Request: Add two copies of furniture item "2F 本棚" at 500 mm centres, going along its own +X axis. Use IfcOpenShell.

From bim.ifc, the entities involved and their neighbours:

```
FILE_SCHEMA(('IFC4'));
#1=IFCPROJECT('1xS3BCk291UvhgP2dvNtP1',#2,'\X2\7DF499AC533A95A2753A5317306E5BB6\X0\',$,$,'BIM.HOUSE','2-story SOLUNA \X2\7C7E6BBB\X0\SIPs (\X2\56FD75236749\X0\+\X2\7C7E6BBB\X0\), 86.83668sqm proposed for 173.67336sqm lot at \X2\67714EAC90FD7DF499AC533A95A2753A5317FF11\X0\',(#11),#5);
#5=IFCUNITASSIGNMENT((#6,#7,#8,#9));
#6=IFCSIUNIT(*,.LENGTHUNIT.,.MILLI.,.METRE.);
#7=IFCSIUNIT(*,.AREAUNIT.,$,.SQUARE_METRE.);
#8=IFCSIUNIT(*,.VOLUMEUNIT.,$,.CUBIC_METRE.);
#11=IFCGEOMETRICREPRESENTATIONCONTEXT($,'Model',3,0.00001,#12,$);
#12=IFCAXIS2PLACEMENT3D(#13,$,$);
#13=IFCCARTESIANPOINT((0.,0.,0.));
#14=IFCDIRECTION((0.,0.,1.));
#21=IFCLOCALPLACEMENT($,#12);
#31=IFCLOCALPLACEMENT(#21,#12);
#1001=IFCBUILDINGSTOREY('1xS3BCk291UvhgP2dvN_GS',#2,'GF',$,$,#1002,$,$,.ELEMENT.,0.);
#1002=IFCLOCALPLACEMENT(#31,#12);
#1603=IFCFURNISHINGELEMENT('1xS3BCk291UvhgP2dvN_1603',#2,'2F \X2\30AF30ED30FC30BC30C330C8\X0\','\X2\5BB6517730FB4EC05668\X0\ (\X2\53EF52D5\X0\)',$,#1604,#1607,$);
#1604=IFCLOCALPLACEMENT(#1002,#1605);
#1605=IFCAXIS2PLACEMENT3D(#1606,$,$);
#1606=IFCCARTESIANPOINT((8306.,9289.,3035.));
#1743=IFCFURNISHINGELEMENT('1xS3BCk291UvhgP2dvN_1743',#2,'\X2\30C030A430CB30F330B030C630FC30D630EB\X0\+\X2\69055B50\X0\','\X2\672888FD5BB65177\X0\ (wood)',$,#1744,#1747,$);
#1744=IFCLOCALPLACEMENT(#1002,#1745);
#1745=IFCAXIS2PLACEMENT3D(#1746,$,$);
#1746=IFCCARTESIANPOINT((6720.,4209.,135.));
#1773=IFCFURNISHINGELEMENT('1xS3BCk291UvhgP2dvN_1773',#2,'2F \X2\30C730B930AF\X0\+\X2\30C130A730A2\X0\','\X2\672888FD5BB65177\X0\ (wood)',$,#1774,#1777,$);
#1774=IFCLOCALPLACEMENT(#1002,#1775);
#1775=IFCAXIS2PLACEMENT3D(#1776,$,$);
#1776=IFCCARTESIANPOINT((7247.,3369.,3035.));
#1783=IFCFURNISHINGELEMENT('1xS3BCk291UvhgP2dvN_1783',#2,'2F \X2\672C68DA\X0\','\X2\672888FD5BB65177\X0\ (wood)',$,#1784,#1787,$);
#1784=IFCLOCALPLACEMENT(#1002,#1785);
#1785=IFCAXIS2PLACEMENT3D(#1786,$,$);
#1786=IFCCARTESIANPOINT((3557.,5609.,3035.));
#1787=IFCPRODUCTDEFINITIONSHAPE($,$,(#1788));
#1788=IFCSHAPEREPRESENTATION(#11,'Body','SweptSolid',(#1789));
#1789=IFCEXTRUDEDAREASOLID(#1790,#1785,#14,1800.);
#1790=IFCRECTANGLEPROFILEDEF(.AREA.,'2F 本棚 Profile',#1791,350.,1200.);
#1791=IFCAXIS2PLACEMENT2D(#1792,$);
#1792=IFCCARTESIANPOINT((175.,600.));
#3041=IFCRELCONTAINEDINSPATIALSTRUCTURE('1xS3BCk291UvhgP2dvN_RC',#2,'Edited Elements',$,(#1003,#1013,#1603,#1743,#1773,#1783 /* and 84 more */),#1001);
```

```python
import ifcopenshell
import ifcopenshell.api.geometry
import ifcopenshell.api.root
import ifcopenshell.util.element
import ifcopenshell.util.placement
import ifcopenshell.util.unit

model = ifcopenshell.open("bim.ifc")
unit_scale = ifcopenshell.util.unit.calculate_unit_scale(model)


def reuse_history(source, copy):
    """copy_class also copies each property set's owner history, people and application; keep the originals."""
    for rel in copy.IsDefinedBy:
        if rel.is_a("IfcRelDefinesByProperties") and (history := rel.RelatingPropertyDefinition.OwnerHistory):
            rel.RelatingPropertyDefinition.OwnerHistory = source.OwnerHistory
            ifcopenshell.util.element.remove_deep2(model, history)


source = model.by_guid("1xS3BCk291UvhgP2dvN_1783")
base = ifcopenshell.util.placement.get_local_placement(source.ObjectPlacement)
step = base[:3, 0] * 0.5 / unit_scale

for i in range(1, 3):
    copy = ifcopenshell.api.root.copy_class(model, product=source)
    copy.Representation = ifcopenshell.util.element.copy_deep(
        model, source.Representation, exclude=["IfcGeometricRepresentationContext", "IfcRepresentationMap"]
    )
    reuse_history(source, copy)
    matrix = base.copy()
    matrix[:3, 3] += i * step
    print("added at", matrix[:3, 3].round(3) + 0.0)
    ifcopenshell.api.geometry.edit_object_placement(model, product=copy, matrix=matrix, is_si=False)

model.write("bim_edited.ifc")
```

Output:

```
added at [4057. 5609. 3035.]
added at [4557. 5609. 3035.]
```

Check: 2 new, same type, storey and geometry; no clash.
